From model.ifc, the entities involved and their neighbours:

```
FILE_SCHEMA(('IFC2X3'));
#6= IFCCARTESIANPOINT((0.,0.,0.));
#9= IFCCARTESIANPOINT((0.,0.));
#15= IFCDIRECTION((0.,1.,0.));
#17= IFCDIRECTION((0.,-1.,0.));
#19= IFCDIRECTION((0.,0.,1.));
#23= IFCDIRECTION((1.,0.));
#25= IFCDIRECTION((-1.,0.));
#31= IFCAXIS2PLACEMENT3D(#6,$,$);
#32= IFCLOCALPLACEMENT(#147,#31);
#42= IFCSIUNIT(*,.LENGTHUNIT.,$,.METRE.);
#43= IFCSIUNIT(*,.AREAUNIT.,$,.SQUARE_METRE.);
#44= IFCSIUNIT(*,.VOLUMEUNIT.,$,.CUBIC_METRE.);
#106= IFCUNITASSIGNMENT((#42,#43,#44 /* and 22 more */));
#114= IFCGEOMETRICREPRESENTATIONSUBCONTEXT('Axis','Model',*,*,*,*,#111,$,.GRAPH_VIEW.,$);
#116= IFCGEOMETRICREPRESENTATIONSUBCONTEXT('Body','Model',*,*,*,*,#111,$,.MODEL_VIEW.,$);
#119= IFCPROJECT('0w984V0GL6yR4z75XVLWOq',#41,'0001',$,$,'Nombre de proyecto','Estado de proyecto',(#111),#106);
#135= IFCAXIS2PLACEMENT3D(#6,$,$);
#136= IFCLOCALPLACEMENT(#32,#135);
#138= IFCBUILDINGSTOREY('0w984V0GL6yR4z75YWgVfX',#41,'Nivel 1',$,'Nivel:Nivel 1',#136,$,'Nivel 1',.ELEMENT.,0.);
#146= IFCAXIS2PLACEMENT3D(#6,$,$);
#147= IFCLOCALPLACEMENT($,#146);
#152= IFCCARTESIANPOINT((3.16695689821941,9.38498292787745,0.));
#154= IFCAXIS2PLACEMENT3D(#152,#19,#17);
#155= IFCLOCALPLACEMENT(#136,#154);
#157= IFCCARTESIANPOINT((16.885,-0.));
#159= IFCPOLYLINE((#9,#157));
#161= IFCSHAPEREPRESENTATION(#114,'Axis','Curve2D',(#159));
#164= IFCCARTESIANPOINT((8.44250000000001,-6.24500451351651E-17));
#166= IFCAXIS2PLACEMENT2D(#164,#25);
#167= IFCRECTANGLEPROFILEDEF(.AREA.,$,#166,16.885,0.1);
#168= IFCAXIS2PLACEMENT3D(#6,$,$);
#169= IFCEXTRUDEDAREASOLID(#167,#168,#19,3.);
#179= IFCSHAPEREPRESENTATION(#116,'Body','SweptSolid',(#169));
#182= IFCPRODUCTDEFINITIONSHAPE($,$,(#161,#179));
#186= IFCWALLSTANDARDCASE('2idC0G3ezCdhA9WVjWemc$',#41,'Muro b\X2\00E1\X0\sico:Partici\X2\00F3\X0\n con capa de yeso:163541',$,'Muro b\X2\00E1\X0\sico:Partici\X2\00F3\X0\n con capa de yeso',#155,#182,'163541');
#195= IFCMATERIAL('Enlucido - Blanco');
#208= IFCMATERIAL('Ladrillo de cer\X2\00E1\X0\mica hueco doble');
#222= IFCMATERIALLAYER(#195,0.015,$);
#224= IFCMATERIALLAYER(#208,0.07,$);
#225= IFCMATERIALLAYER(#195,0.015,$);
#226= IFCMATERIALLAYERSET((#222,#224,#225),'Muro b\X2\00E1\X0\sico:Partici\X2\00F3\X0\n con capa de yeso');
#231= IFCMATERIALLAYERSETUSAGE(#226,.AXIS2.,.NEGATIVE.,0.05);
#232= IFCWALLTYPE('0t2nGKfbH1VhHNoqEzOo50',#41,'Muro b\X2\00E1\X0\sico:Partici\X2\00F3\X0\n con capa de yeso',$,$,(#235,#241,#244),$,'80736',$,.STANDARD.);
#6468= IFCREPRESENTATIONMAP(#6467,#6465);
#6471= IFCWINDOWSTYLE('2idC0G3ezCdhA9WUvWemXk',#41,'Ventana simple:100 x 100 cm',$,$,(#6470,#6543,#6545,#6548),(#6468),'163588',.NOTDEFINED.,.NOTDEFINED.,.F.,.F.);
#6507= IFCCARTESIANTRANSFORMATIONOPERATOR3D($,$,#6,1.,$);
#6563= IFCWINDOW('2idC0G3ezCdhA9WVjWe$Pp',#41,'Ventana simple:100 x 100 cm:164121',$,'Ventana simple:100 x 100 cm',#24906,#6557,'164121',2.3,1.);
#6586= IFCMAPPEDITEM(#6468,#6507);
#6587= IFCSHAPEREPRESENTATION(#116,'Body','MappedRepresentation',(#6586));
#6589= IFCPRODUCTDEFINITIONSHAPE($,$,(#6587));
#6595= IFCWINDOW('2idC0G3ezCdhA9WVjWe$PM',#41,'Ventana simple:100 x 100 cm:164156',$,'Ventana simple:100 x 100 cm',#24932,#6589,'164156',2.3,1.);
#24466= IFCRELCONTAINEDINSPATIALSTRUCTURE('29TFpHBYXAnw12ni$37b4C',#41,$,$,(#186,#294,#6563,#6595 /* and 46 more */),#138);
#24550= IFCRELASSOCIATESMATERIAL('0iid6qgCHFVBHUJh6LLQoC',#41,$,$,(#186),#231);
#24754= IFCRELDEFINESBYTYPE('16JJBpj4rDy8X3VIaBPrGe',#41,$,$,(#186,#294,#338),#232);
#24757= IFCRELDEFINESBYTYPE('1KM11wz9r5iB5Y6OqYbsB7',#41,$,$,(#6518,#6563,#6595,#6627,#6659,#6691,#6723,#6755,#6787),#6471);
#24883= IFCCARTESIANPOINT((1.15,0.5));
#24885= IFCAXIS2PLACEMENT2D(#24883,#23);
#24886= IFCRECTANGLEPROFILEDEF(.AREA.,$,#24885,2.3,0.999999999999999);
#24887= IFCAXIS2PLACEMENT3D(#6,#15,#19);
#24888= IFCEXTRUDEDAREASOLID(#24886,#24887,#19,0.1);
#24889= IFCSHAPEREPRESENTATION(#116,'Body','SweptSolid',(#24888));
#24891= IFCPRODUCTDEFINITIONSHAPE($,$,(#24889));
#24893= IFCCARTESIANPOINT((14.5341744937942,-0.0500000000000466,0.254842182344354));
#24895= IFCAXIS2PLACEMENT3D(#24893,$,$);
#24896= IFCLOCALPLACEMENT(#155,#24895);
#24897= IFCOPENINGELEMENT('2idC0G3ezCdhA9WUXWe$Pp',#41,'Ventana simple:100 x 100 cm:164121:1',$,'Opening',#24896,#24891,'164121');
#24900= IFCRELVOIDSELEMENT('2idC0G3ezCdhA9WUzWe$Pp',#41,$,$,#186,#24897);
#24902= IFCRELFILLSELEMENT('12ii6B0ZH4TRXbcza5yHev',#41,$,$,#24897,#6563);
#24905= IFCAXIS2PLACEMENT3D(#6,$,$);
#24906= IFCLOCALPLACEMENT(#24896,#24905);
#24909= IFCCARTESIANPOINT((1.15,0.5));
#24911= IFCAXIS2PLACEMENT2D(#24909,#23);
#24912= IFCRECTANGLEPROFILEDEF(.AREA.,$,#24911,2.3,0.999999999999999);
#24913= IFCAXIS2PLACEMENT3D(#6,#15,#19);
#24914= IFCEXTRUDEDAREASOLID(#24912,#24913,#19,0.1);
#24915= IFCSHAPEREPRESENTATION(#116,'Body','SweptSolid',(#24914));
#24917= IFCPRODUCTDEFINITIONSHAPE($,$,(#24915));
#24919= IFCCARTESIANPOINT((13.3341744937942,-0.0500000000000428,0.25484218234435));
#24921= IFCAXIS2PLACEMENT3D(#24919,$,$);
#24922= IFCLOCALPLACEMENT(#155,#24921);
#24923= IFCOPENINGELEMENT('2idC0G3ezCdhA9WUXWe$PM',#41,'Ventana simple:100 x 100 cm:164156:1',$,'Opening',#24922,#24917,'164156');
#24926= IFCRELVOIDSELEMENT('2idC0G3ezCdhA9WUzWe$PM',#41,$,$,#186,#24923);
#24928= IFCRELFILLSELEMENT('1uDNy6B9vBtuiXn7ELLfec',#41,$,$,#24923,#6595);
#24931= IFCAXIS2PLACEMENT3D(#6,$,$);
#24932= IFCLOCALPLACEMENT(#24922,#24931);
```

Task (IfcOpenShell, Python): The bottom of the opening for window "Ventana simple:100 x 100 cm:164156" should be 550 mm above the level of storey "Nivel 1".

```python
import numpy as np
import ifcopenshell
import ifcopenshell.api.geometry
import ifcopenshell.geom
import ifcopenshell.util.element
import ifcopenshell.util.placement
import ifcopenshell.util.shape
import ifcopenshell.util.unit

model = ifcopenshell.open("model.ifc")
unit_scale = ifcopenshell.util.unit.calculate_unit_scale(model)

window = model.by_id(6595)
opening = window.FillsVoids[0].RelatingOpeningElement
storey = ifcopenshell.util.element.get_container(window, ifc_class="IfcBuildingStorey")
level = ifcopenshell.util.placement.get_local_placement(storey.ObjectPlacement)[2, 3]

# The opening's origin need not be at the sill, so measure its lowest point.
shape = ifcopenshell.geom.create_shape(ifcopenshell.geom.settings(), opening)
bottom = ifcopenshell.util.shape.get_shape_bottom_elevation(shape, shape.geometry) / unit_scale
dz = level + 0.55 / unit_scale - bottom

shift = np.array([0.0, 0.0, dz])
# The window is placed relative to its opening, so it follows when the opening moves.
matrix = ifcopenshell.util.placement.get_local_placement(opening.ObjectPlacement)
matrix[:3, 3] += shift
ifcopenshell.api.geometry.edit_object_placement(
    model, product=opening, matrix=matrix, is_si=False, should_transform_children=True
)

print(f"moved by {dz * unit_scale:+.3f} m")

model.write("model_updated.ifc")
```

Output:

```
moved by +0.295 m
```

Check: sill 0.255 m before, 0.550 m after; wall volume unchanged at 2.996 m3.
